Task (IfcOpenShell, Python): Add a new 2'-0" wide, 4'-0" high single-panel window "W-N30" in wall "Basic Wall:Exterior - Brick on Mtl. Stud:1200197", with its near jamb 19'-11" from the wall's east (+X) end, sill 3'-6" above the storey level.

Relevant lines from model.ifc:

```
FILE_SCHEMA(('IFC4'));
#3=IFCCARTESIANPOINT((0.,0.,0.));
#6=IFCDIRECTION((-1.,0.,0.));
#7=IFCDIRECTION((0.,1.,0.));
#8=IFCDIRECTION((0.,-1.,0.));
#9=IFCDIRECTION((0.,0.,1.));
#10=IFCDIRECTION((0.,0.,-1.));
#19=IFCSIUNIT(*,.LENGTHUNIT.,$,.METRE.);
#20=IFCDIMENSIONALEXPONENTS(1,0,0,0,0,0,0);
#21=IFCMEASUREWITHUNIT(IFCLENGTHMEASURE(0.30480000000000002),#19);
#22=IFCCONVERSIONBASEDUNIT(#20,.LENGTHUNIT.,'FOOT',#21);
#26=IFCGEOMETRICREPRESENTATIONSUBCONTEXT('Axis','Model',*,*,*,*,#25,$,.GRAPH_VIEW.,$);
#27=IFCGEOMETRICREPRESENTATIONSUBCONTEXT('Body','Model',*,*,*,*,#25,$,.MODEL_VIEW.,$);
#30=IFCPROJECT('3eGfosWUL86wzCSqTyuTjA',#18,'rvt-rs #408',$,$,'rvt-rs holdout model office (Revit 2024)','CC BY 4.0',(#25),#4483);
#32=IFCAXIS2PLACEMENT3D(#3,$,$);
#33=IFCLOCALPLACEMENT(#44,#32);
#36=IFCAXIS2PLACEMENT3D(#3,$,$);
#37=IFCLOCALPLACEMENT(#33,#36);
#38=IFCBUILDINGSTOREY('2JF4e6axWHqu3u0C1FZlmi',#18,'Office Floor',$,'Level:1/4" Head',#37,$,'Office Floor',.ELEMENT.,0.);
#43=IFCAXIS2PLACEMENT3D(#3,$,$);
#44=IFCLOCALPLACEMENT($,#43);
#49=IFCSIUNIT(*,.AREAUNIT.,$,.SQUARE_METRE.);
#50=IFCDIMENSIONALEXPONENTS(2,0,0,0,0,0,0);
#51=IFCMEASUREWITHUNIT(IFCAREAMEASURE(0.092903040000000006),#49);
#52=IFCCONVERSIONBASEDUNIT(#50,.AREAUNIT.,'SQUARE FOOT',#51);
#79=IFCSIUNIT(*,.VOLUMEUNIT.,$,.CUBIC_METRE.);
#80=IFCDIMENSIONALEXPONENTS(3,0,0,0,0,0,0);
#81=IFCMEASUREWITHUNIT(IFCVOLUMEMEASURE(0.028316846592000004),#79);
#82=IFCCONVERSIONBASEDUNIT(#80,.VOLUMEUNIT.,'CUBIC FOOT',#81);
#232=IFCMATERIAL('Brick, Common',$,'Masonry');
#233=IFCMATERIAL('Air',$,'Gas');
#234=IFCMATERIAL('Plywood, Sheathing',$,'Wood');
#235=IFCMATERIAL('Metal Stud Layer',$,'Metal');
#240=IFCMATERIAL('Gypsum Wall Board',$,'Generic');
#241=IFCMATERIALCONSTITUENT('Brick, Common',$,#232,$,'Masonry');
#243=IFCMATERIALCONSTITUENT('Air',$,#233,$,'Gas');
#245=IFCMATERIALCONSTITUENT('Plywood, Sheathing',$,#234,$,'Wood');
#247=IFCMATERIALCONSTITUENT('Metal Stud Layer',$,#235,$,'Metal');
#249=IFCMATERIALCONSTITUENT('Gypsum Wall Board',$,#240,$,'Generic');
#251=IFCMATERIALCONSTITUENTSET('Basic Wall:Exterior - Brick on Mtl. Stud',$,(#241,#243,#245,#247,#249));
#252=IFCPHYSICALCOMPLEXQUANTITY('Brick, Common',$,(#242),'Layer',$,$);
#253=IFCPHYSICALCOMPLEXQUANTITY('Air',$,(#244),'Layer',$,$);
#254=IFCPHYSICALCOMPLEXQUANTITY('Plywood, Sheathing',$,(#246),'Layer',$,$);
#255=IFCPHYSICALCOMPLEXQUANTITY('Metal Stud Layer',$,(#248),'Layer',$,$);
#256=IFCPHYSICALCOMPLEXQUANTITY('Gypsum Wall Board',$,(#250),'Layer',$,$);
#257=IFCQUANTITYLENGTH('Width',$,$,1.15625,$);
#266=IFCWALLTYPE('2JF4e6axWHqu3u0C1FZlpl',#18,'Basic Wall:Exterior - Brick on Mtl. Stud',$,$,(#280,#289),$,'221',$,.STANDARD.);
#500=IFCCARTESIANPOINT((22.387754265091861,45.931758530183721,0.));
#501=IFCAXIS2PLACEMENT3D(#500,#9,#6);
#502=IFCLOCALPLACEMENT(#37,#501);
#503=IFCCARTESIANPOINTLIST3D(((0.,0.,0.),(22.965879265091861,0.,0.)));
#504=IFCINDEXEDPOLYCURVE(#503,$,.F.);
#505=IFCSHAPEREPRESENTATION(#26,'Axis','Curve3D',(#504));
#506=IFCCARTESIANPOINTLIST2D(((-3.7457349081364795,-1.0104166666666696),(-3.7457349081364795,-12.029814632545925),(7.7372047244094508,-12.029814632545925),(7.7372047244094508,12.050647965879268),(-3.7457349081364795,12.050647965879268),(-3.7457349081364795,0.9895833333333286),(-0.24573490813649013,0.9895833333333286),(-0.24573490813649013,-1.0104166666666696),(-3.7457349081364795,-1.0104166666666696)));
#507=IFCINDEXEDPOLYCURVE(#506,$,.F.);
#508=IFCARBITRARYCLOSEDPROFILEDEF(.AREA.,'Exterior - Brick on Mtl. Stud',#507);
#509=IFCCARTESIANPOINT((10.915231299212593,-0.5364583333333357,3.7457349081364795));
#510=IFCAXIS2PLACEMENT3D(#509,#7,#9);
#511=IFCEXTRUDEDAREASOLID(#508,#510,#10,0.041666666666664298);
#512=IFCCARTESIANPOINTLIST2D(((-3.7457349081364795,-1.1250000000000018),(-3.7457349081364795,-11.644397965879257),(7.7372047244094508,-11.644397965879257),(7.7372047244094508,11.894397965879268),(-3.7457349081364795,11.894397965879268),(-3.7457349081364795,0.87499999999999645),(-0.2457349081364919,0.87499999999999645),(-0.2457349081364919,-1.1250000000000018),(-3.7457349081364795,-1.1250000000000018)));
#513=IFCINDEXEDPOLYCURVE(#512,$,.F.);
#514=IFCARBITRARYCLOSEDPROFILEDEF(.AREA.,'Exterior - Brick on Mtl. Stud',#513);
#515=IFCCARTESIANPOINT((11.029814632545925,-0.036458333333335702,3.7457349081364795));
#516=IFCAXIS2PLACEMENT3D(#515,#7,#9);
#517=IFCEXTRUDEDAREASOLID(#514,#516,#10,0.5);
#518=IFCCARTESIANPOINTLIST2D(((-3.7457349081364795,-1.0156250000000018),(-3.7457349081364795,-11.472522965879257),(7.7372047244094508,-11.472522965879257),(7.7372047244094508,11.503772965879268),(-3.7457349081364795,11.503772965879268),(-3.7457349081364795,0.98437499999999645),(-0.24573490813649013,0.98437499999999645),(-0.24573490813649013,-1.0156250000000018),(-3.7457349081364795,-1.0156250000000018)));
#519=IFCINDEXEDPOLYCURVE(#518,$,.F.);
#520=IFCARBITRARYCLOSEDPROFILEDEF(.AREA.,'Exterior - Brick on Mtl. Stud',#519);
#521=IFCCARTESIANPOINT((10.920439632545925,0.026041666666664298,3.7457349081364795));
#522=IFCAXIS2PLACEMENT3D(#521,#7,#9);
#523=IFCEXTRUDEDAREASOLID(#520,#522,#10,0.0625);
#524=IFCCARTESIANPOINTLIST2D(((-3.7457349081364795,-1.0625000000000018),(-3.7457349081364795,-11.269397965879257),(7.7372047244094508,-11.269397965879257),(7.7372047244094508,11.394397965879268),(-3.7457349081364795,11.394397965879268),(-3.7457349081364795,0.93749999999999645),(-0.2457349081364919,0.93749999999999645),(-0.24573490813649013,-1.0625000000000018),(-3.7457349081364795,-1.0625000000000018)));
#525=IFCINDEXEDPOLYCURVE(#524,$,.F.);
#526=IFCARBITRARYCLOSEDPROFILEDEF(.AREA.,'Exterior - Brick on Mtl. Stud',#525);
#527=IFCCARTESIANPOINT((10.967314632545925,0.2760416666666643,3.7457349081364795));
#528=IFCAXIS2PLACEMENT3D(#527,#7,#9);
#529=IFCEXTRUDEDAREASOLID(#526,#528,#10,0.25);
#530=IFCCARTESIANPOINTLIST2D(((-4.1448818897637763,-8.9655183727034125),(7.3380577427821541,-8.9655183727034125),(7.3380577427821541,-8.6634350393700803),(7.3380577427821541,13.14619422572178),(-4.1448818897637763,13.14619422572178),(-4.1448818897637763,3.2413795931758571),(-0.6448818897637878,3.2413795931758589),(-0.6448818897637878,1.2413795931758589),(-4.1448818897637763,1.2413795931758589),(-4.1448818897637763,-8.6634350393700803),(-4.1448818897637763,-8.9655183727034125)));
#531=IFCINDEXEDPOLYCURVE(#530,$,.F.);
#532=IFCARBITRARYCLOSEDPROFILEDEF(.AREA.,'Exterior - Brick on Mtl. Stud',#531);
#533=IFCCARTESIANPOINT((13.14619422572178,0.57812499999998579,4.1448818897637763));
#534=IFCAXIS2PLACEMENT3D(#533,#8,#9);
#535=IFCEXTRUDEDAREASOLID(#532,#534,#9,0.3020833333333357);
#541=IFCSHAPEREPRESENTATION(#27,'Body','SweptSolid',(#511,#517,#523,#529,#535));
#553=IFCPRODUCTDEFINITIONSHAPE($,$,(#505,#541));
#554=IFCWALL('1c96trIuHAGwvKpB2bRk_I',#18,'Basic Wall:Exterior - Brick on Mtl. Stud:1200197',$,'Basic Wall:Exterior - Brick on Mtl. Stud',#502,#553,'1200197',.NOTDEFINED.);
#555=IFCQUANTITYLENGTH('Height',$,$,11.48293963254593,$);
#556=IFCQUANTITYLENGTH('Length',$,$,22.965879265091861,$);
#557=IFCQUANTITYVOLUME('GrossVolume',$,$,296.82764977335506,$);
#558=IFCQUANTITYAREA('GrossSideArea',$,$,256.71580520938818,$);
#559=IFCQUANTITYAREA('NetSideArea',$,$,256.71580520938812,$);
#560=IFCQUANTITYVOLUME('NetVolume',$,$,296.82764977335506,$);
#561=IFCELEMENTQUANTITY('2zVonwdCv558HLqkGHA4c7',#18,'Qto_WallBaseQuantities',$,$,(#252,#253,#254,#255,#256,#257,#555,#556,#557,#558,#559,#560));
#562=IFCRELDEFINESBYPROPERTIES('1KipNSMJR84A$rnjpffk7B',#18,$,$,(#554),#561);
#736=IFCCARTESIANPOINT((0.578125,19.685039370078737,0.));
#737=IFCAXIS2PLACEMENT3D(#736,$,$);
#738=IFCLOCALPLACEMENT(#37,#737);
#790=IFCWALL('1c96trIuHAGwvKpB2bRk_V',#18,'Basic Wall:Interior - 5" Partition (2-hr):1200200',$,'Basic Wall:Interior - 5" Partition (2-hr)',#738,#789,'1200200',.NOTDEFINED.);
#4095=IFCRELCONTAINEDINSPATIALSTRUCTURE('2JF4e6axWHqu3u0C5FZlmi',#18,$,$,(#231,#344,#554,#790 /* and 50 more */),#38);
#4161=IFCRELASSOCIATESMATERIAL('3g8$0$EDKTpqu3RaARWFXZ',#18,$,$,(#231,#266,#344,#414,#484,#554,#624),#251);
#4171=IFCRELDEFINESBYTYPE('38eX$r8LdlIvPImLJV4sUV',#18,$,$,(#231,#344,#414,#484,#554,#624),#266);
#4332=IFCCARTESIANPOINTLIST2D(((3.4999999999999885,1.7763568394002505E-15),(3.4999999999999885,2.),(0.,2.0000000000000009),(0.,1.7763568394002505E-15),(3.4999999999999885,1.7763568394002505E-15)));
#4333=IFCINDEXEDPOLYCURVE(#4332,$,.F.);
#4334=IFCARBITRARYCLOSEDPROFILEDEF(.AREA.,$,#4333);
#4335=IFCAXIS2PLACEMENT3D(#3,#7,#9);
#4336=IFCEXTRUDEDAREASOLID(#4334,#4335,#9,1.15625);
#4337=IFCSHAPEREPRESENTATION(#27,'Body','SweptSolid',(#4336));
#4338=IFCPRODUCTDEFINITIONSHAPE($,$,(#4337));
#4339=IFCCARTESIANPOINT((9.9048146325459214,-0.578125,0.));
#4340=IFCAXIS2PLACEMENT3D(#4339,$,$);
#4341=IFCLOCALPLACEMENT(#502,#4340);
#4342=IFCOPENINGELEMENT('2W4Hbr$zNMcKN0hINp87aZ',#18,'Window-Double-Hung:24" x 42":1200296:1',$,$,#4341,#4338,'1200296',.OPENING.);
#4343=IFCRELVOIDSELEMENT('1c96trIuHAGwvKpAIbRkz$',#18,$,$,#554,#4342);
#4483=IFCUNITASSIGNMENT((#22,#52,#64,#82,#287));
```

```python
import numpy as np
import ifcopenshell
import ifcopenshell.api.feature
import ifcopenshell.api.geometry
import ifcopenshell.api.pset
import ifcopenshell.api.root
import ifcopenshell.api.spatial
import ifcopenshell.geom
import ifcopenshell.util.element
import ifcopenshell.util.placement
import ifcopenshell.util.representation
import ifcopenshell.util.shape
import ifcopenshell.util.unit

model = ifcopenshell.open("model.ifc")
unit_scale = ifcopenshell.util.unit.calculate_unit_scale(model)
area_scale = ifcopenshell.util.unit.calculate_unit_scale(model, "AREAUNIT")
volume_scale = ifcopenshell.util.unit.calculate_unit_scale(model, "VOLUMEUNIT")
settings = ifcopenshell.geom.settings()


def volume(element):
    """Net volume in cubic metres, openings subtracted."""
    shape = ifcopenshell.geom.create_shape(settings, element)
    return ifcopenshell.util.shape.get_volume(shape.geometry)


wall = model.by_guid("1c96trIuHAGwvKpB2bRk_I")
storey = ifcopenshell.util.element.get_container(wall, ifc_class="IfcBuildingStorey")
context = ifcopenshell.util.representation.get_context(model, "Model", "Body", "MODEL_VIEW")
before = volume(wall)

width, height, from_end, sill = 0.6096, 1.2192, 6.0706, 1.0668  # metres

# The wall runs along its own X axis, and the end named is its -X end.
wall_shape = ifcopenshell.geom.create_shape(settings, wall)
x, y, z = ifcopenshell.util.shape.get_vertices(wall_shape.geometry).T
start = x.min() + from_end
face, thickness = float(y.min()), float(y.max() - y.min())
wall_matrix = ifcopenshell.util.placement.get_local_placement(wall.ObjectPlacement)
level = ifcopenshell.util.placement.get_local_placement(storey.ObjectPlacement)[2, 3]


def in_wall(x, y):
    """Placement at x, y metres in the wall's axes, at sill height."""
    matrix = wall_matrix.copy()
    matrix[:, 3] = wall_matrix @ np.array([x / unit_scale, y / unit_scale, 0.0, 1.0])
    matrix[2, 3] = level + sill / unit_scale
    return matrix


# Opening: a box that overshoots both wall faces by 50 mm.
opening = ifcopenshell.api.root.create_entity(model, ifc_class="IfcOpeningElement", predefined_type="OPENING")
box = ifcopenshell.api.geometry.add_wall_representation(
    model, context=context, length=width, height=height, thickness=thickness + 0.1
)
ifcopenshell.api.geometry.assign_representation(model, product=opening, representation=box)
ifcopenshell.api.geometry.edit_object_placement(model, product=opening, matrix=in_wall(start, face - 0.05), is_si=False)
ifcopenshell.api.feature.add_feature(model, feature=opening, element=wall)

window = ifcopenshell.api.root.create_entity(model, ifc_class="IfcWindow", name="W-N30", predefined_type="WINDOW")
window.OverallWidth, window.OverallHeight = width / unit_scale, height / unit_scale
window.PartitioningType = "SINGLE_PANEL"
body = ifcopenshell.api.geometry.add_window_representation(
    model,
    context=context,
    overall_width=window.OverallWidth,
    overall_height=window.OverallHeight,
    partition_type="SINGLE_PANEL",
)
ifcopenshell.api.geometry.assign_representation(model, product=window, representation=body)
ifcopenshell.api.spatial.assign_container(model, products=[window], relating_structure=storey)
ifcopenshell.api.feature.add_filling(model, opening=opening, element=window)

# Centre the window in the wall's thickness.
ifcopenshell.api.geometry.edit_object_placement(model, product=window, matrix=in_wall(start, face), is_si=False)
window_shape = ifcopenshell.geom.create_shape(settings, window)
depth = ifcopenshell.util.shape.get_vertices(window_shape.geometry)[:, 1]
offset = face + thickness / 2 - (depth.min() + depth.max()) / 2
ifcopenshell.api.geometry.edit_object_placement(model, product=window, matrix=in_wall(start, offset), is_si=False)

after = volume(wall)

# Update the wall's stored quantities.
qto = model.by_id(ifcopenshell.util.element.get_pset(wall, "Qto_WallBaseQuantities", should_inherit=False)["id"])
ifcopenshell.api.pset.edit_qto(model, qto=qto, properties={
    "NetSideArea": after / thickness / area_scale,
    "NetVolume": after / volume_scale,
})

print(f"wall volume {before:.3f} -> {after:.3f} m3")

model.write("model_rev.ifc")
```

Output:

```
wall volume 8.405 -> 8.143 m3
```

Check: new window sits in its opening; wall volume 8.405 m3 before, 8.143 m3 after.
